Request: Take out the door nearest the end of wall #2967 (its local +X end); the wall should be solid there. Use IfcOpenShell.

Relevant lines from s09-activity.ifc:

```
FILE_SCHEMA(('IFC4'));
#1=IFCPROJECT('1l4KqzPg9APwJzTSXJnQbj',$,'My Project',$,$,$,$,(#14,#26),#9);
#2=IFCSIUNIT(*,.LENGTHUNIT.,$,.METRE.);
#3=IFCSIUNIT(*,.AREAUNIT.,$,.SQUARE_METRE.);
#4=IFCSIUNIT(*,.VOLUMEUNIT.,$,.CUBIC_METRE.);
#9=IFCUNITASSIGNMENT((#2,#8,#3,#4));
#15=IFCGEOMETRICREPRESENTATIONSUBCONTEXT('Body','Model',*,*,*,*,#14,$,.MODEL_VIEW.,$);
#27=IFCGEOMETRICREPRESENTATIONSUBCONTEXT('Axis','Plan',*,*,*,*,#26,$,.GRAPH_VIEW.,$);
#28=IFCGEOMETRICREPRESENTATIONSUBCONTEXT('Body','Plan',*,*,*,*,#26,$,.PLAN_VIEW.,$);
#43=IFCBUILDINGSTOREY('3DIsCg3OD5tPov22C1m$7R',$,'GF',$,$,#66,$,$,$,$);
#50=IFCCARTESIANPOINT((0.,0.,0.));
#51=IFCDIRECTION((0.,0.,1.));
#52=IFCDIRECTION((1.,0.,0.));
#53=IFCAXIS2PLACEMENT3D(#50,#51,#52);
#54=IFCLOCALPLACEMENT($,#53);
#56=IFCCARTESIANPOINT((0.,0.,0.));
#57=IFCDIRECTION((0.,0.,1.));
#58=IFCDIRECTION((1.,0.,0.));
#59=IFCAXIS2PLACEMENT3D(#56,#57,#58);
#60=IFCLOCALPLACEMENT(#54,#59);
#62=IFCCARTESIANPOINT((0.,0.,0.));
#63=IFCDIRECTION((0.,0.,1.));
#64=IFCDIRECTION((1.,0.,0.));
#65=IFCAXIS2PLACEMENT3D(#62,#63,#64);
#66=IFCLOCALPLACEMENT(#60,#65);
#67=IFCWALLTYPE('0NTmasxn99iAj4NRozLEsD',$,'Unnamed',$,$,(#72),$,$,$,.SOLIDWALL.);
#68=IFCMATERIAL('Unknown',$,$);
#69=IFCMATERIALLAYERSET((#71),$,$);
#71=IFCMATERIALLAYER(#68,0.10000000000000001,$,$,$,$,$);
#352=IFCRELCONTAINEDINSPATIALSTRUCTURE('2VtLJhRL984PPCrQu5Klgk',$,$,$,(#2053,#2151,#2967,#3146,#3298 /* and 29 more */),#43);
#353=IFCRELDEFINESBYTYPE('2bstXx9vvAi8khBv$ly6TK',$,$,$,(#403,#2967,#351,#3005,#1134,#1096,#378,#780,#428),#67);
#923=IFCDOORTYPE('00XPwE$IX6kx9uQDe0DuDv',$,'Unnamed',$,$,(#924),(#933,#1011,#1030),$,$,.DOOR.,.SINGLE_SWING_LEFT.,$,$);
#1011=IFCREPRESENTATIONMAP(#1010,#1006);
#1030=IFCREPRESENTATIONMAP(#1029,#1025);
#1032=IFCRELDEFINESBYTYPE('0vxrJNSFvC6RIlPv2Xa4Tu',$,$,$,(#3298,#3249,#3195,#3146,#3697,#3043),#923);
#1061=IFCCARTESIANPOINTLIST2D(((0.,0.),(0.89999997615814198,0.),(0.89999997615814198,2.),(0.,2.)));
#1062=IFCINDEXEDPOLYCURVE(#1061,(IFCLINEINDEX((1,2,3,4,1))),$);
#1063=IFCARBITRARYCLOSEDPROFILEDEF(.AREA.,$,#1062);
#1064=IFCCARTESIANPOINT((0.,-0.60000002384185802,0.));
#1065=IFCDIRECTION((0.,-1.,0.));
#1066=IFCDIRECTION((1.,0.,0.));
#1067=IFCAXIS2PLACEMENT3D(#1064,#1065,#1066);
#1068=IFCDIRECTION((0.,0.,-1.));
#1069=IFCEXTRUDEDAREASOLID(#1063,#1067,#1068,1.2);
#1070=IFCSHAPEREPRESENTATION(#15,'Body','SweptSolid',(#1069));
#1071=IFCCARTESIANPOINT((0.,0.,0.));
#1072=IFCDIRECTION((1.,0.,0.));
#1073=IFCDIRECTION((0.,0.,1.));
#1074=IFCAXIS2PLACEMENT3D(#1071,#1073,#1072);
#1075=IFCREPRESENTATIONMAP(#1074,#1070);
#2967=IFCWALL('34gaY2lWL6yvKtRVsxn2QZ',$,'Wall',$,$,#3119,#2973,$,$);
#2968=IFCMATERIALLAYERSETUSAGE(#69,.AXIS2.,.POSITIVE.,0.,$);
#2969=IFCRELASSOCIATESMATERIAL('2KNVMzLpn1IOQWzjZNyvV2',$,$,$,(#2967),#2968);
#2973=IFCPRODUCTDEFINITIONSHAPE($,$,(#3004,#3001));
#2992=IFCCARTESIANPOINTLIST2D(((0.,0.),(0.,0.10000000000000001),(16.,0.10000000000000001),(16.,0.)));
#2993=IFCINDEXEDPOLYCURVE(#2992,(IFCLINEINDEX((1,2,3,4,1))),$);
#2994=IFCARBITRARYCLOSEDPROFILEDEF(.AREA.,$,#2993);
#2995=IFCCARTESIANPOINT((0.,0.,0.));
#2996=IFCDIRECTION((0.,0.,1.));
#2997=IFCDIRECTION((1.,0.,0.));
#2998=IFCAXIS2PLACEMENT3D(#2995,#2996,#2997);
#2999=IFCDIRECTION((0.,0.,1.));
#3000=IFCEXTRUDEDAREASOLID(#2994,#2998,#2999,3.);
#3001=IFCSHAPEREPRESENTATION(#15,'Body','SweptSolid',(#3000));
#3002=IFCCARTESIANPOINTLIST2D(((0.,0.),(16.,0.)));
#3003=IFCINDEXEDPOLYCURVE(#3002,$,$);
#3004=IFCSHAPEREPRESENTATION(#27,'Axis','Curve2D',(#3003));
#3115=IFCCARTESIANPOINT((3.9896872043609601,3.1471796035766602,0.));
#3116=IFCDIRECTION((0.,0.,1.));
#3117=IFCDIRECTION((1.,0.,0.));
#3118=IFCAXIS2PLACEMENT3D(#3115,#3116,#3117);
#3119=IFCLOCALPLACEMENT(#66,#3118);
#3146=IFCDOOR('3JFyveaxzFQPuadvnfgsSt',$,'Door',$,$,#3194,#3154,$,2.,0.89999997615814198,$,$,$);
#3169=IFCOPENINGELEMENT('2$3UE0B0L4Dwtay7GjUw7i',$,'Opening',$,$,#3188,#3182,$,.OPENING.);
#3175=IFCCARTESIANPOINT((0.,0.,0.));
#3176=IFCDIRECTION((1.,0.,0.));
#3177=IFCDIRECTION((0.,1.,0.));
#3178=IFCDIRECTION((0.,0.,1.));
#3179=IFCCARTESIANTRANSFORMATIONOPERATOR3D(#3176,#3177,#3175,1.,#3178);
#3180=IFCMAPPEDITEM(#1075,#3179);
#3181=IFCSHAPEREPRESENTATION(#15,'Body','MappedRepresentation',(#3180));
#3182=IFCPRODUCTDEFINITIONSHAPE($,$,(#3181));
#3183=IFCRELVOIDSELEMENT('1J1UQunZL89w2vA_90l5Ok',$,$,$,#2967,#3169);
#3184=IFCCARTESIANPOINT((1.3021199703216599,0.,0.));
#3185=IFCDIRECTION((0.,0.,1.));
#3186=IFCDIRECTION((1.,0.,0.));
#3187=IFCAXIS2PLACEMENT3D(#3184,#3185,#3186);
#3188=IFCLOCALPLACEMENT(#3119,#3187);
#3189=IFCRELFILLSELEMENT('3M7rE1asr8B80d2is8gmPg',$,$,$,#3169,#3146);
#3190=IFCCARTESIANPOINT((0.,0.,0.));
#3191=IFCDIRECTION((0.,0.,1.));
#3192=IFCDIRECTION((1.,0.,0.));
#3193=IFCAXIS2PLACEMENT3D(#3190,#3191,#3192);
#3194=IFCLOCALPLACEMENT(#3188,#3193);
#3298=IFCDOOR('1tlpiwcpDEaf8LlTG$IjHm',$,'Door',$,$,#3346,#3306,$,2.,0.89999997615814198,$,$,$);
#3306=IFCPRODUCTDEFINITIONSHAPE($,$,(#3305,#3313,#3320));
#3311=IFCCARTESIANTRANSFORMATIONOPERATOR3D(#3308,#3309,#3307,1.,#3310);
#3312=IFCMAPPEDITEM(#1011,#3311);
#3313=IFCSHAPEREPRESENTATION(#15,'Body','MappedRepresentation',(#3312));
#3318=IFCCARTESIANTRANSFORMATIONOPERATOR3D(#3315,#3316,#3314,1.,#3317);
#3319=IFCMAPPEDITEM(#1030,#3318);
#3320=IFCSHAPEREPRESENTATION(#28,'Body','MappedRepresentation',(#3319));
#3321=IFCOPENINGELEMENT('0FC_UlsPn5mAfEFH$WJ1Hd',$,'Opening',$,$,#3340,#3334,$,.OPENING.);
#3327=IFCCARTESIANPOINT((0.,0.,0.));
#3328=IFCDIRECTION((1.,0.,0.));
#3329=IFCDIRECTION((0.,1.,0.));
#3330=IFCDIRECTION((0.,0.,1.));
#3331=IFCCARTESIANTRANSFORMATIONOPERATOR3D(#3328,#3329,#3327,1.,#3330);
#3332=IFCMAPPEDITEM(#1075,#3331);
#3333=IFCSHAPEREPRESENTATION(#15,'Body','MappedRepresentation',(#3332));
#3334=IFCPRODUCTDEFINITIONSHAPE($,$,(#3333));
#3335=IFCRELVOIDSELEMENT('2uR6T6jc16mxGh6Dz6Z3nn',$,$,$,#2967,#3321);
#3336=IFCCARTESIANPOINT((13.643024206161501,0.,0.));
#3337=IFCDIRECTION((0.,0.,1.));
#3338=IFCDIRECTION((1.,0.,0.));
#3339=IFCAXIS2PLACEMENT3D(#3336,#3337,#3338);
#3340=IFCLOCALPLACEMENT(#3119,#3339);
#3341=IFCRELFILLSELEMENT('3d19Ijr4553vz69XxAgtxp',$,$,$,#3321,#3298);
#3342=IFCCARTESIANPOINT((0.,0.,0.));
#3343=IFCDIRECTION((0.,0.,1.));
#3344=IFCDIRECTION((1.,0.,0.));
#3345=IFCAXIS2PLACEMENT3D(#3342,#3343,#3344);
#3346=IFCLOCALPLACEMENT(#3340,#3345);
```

```python
import ifcopenshell
import ifcopenshell.api.feature
import ifcopenshell.api.root
import ifcopenshell.geom
import ifcopenshell.util.shape

model = ifcopenshell.open("s09-activity.ifc")
settings = ifcopenshell.geom.settings()


def volume(element):
    """Net volume in cubic metres, openings subtracted."""
    shape = ifcopenshell.geom.create_shape(settings, element)
    return ifcopenshell.util.shape.get_volume(shape.geometry)


door = model.by_id(3298)
opening = door.FillsVoids[0].RelatingOpeningElement
wall = opening.VoidsElements[0].RelatingBuildingElement
before = volume(wall)

ifcopenshell.api.root.remove_product(model, product=door)
ifcopenshell.api.feature.remove_feature(model, feature=opening)

after = volume(wall)

print(f"wall volume {before:.3f} -> {after:.3f} m3")

model.write("s09-activity_v2.ifc")
```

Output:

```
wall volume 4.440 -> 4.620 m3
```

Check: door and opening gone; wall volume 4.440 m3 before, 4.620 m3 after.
